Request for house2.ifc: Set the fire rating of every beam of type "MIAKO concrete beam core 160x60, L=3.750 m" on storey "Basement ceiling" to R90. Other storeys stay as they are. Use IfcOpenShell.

First a look at what the model holds.

```python
import ifcopenshell
import ifcopenshell.util.element

model = ifcopenshell.open("house2.ifc")
print(model.schema)
storey = next(s for s in model.by_type("IfcBuildingStorey") if s.Name == "Basement ceiling")
beams = [e for e in ifcopenshell.util.element.get_decomposition(storey) if e.is_a("IfcBeam")]
seen = {}
for e in beams:
    element_type = ifcopenshell.util.element.get_type(e)
    key = (element_type.Name if element_type != e and element_type else None, ifcopenshell.util.element.get_pset(e, "Pset_BeamCommon", "FireRating"))
    seen[key] = seen.get(key, 0) + 1
for (name, value), count in sorted(seen.items(), key=str):
    print(count, "x", name, "|", value)
```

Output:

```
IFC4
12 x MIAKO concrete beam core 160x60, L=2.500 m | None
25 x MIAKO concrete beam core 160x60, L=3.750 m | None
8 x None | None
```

```python
import ifcopenshell
import ifcopenshell.api.pset
import ifcopenshell.util.element

model = ifcopenshell.open("house2.ifc")

storey = next(s for s in model.by_type("IfcBuildingStorey") if s.Name == "Basement ceiling")
beams = [e for e in ifcopenshell.util.element.get_decomposition(storey) if e.is_a("IfcBeam")]

count = 0
for e in beams:
    element_type = ifcopenshell.util.element.get_type(e)
    if element_type in (None, e) or element_type.Name != "MIAKO concrete beam core 160x60, L=3.750 m":
        continue
    # add_pset returns the element's existing set when there is one.
    pset = ifcopenshell.api.pset.add_pset(model, product=e, name="Pset_BeamCommon")
    ifcopenshell.api.pset.edit_pset(model, pset=pset, properties={"FireRating": "R90"})
    count += 1

print(count, "beams updated")

model.write("house2_edited.ifc")
```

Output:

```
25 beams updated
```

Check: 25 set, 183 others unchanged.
